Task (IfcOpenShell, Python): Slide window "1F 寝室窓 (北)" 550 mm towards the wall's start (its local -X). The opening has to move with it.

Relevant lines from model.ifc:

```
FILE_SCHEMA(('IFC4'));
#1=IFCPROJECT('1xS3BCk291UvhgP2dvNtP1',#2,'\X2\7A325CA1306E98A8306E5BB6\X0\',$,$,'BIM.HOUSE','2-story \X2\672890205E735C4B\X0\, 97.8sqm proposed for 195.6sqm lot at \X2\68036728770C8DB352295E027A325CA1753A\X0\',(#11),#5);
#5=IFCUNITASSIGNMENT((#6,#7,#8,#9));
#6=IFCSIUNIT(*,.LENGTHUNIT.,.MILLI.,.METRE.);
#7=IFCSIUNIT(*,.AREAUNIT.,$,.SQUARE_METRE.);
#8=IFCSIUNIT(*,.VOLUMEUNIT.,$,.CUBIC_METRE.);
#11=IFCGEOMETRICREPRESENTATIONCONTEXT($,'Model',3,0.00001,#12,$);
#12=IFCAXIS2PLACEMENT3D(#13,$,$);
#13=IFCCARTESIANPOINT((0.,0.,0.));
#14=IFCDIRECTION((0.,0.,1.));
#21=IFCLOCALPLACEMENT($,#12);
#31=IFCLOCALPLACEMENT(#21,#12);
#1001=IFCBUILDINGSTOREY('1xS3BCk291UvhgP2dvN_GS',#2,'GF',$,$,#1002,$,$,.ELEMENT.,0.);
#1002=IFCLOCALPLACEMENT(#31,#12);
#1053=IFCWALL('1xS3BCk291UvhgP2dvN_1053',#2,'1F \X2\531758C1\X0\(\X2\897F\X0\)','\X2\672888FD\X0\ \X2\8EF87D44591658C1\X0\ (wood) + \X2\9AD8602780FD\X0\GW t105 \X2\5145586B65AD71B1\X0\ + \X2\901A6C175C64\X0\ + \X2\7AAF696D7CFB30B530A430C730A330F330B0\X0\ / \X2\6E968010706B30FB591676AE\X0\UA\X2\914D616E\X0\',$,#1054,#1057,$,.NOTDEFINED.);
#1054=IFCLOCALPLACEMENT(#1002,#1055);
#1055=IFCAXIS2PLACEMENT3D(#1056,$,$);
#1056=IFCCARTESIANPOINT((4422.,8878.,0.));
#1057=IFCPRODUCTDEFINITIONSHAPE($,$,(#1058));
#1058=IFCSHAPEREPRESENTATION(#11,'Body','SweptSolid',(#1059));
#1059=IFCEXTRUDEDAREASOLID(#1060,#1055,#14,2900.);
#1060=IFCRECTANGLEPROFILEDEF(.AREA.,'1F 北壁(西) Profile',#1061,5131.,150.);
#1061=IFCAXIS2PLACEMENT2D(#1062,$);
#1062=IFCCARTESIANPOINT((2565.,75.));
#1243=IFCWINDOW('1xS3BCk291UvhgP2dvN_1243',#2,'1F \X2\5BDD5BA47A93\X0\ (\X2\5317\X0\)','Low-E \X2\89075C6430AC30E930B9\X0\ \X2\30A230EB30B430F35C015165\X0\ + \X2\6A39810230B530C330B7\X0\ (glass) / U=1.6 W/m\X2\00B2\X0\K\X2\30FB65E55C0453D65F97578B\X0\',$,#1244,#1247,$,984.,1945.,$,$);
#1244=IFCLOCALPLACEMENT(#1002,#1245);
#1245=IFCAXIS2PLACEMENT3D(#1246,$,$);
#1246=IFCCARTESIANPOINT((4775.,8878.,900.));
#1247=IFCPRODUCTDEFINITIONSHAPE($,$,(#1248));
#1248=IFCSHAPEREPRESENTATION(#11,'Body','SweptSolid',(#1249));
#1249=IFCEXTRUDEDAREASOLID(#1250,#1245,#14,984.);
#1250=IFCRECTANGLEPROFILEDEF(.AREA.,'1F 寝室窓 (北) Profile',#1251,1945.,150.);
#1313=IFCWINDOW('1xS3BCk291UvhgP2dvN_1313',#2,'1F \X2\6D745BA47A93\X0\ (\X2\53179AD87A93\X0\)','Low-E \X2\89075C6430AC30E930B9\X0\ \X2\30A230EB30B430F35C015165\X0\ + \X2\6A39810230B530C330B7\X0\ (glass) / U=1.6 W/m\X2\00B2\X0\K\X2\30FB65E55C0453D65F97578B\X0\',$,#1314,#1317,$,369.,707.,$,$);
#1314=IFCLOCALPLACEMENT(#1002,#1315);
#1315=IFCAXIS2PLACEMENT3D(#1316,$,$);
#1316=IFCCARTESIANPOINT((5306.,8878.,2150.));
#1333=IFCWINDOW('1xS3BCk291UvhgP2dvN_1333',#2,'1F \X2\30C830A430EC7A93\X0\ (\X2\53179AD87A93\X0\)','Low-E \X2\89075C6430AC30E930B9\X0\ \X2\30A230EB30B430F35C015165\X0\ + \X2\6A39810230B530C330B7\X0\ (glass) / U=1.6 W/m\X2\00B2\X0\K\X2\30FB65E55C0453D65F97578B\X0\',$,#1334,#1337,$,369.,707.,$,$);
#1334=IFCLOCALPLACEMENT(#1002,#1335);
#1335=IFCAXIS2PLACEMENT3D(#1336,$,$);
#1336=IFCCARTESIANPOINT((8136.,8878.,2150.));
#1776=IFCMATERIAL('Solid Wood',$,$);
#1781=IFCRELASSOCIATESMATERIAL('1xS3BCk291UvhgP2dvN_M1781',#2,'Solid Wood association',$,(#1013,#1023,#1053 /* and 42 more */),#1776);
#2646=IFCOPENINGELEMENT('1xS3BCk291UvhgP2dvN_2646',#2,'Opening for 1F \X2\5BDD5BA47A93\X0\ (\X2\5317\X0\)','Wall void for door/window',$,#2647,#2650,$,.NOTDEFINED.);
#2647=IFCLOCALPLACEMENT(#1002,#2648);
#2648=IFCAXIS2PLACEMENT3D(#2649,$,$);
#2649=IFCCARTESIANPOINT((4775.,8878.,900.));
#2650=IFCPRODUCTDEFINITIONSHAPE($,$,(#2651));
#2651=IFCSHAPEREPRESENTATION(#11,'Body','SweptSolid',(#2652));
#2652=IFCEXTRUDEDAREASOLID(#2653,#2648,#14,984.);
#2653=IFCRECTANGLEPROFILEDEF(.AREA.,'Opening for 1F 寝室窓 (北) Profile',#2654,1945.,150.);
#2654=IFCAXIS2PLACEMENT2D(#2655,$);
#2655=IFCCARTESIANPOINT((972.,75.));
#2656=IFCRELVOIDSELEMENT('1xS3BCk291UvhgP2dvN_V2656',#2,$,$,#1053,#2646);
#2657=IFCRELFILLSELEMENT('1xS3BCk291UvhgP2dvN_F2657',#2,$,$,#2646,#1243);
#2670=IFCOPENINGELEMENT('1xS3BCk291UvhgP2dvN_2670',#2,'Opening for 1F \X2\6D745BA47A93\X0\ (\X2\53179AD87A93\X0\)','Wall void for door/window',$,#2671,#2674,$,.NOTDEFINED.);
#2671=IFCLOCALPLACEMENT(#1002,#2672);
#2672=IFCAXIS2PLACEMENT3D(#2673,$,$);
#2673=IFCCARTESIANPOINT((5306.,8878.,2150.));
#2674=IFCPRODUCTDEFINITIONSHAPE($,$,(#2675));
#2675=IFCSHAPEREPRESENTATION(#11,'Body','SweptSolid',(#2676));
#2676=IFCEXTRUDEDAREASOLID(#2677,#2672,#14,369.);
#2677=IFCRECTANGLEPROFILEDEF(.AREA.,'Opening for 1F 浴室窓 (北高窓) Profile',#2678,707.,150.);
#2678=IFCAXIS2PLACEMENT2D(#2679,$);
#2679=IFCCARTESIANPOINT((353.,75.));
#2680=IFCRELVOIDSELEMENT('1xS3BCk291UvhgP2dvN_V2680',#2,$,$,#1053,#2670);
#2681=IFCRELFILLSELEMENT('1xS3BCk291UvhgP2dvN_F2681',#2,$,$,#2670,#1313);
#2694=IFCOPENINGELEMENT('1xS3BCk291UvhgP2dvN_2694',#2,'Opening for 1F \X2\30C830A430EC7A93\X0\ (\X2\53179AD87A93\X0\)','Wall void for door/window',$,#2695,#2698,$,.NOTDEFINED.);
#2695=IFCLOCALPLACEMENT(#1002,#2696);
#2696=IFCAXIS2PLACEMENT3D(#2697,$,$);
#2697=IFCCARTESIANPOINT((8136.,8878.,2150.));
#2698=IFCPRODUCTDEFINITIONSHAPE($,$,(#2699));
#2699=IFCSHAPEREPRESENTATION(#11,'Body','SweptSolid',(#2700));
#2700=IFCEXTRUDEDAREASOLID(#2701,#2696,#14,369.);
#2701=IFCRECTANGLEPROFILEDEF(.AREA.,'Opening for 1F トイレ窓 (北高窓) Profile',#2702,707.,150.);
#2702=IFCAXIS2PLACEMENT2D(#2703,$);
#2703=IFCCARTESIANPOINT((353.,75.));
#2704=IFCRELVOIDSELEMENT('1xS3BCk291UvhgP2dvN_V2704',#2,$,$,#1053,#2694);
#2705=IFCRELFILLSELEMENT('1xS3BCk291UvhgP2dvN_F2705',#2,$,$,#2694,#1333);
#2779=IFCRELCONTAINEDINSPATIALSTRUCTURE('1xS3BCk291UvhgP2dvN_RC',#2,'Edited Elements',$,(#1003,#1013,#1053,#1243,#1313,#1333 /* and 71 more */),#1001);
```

```python
import ifcopenshell
import ifcopenshell.api.geometry
import ifcopenshell.util.placement

model = ifcopenshell.open("model.ifc")

window = model.by_guid("1xS3BCk291UvhgP2dvN_1243")
opening = window.FillsVoids[0].RelatingOpeningElement
wall = opening.VoidsElements[0].RelatingBuildingElement

wall_matrix = ifcopenshell.util.placement.get_local_placement(wall.ObjectPlacement)
shift = wall_matrix[:3, 0] * -550.0
before = ifcopenshell.util.placement.get_local_placement(window.ObjectPlacement)[:3, 3].copy()

# The window is not placed relative to its opening, so move both.
for product in (opening, window):
    matrix = ifcopenshell.util.placement.get_local_placement(product.ObjectPlacement)
    matrix[:3, 3] += shift
    ifcopenshell.api.geometry.edit_object_placement(model, product=product, matrix=matrix, is_si=False)

after = ifcopenshell.util.placement.get_local_placement(window.ObjectPlacement)[:3, 3]
print("window moved by", (after - before).round(3) + 0.0)

model.write("model_updated.ifc")
```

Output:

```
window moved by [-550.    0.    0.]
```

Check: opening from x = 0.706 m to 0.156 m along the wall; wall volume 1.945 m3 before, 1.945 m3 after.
